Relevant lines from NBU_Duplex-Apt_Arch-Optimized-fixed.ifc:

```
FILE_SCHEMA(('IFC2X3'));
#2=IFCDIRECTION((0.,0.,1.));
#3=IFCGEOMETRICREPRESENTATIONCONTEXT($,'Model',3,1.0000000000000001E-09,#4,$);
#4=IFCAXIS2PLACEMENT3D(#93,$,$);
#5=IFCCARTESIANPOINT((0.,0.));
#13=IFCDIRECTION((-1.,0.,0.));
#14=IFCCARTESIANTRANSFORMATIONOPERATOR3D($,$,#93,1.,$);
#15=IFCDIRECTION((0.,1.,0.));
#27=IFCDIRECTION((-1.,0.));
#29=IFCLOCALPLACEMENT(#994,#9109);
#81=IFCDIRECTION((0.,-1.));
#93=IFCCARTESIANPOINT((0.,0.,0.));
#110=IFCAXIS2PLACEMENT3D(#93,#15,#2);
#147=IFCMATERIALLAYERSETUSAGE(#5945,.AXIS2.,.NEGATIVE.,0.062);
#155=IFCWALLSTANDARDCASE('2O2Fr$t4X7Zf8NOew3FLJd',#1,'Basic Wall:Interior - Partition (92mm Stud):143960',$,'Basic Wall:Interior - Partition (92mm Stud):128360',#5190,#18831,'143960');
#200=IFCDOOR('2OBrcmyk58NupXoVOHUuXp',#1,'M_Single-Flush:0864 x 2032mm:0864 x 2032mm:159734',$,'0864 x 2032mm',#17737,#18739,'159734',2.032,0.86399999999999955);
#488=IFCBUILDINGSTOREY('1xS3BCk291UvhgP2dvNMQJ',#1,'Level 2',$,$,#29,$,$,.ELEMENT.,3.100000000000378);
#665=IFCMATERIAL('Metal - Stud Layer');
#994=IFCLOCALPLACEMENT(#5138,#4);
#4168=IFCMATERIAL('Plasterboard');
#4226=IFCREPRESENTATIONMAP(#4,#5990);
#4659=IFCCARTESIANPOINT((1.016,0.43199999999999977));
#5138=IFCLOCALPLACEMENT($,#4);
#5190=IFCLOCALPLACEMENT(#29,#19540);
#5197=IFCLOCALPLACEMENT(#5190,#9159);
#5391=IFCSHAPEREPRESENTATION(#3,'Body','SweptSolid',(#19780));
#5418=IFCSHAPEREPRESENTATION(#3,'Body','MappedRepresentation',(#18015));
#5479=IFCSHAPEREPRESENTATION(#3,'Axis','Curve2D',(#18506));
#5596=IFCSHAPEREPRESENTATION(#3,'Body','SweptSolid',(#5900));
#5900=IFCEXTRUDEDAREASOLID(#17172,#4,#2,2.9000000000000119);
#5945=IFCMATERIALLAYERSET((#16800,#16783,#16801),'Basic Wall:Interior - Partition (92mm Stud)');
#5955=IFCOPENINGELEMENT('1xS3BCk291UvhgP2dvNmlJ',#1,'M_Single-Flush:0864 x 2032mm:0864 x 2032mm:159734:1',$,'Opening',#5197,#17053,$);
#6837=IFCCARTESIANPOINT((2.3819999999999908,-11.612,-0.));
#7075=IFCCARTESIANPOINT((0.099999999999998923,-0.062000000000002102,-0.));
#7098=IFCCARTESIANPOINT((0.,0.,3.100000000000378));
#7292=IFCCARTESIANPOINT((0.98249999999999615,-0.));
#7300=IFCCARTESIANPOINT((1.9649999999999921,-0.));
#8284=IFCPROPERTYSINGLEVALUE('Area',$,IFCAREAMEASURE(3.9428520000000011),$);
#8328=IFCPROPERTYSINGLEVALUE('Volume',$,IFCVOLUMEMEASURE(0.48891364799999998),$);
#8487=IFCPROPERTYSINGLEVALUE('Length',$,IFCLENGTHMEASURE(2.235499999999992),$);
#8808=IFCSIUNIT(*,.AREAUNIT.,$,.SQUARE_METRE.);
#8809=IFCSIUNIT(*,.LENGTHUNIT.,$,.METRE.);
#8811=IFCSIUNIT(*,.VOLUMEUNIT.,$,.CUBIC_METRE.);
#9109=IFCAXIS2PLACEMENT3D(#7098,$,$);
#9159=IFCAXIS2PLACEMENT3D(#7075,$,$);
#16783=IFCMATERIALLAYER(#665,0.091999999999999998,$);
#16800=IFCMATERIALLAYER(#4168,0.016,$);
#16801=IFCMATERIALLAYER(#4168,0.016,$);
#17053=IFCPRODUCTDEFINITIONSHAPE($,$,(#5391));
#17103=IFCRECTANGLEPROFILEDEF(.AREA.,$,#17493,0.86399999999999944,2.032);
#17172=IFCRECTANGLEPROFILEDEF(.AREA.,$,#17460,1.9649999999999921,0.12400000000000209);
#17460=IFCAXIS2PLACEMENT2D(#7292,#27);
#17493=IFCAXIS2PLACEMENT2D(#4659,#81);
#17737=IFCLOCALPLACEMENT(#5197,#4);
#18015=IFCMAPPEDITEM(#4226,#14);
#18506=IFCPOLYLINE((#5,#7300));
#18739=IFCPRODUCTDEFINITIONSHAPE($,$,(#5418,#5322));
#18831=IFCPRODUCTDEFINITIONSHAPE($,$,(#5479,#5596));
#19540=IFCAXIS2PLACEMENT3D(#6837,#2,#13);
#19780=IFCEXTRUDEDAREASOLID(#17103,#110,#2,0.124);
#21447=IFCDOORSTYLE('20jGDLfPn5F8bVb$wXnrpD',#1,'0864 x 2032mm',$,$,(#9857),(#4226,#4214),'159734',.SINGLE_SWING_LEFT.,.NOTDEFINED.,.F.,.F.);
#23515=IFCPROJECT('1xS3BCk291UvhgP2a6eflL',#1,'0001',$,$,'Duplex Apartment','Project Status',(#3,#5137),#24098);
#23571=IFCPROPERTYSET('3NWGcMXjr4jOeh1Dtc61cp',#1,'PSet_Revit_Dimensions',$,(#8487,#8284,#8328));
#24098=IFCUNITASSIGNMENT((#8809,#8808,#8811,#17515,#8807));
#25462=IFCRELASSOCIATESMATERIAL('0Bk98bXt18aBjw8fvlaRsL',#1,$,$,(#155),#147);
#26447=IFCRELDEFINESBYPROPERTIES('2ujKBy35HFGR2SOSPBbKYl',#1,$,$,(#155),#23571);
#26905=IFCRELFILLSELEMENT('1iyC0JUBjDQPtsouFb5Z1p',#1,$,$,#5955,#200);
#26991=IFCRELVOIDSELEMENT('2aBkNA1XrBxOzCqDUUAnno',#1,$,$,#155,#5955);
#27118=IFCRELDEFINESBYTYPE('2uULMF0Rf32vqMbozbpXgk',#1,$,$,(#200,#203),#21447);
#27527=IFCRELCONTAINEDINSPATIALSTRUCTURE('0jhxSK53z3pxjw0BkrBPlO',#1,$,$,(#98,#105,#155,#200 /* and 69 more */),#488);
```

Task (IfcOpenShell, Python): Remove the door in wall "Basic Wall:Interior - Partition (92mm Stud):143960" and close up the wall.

```python
import ifcopenshell
import ifcopenshell.api.feature
import ifcopenshell.api.pset
import ifcopenshell.api.root
import ifcopenshell.geom
import ifcopenshell.util.element
import ifcopenshell.util.shape
import ifcopenshell.util.unit

model = ifcopenshell.open("NBU_Duplex-Apt_Arch-Optimized-fixed.ifc")
area_scale = ifcopenshell.util.unit.calculate_unit_scale(model, "AREAUNIT")
volume_scale = ifcopenshell.util.unit.calculate_unit_scale(model, "VOLUMEUNIT")
settings = ifcopenshell.geom.settings()


def volume(element):
    """Net volume in cubic metres, openings subtracted."""
    shape = ifcopenshell.geom.create_shape(settings, element)
    return ifcopenshell.util.shape.get_volume(shape.geometry)


door = model.by_guid("2OBrcmyk58NupXoVOHUuXp")
opening = door.FillsVoids[0].RelatingOpeningElement
wall = opening.VoidsElements[0].RelatingBuildingElement
before = volume(wall)

ifcopenshell.api.root.remove_product(model, product=door)
ifcopenshell.api.feature.remove_feature(model, feature=opening)

after = volume(wall)
thickness = 0.124  # wall thickness in metres

# Update the wall's stored quantities.
pset = model.by_id(ifcopenshell.util.element.get_pset(wall, "PSet_Revit_Dimensions", should_inherit=False)["id"])
ifcopenshell.api.pset.edit_pset(model, pset=pset, properties={
    "Area": model.create_entity("IfcAreaMeasure", after / thickness / area_scale),
    "Volume": model.create_entity("IfcVolumeMeasure", after / volume_scale),
})

print(f"wall volume {before:.3f} -> {after:.3f} m3")

model.write("NBU_Duplex-Apt_Arch-Optimized-fixed_edited.ifc")
```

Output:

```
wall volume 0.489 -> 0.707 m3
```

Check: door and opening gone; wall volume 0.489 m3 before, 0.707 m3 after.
